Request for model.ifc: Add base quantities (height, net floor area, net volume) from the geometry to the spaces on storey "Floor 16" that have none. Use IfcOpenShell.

First a look at what the model holds.

```python
import ifcopenshell
import ifcopenshell.util.element
import ifcopenshell.util.unit

model = ifcopenshell.open("model.ifc")
print(model.schema)
for unit_type in ("LENGTHUNIT", "AREAUNIT", "VOLUMEUNIT"):
    print(unit_type, ifcopenshell.util.unit.calculate_unit_scale(model, unit_type))
storey = next(s for s in model.by_type("IfcBuildingStorey") if s.Name == "Floor 16")
spaces = [e for e in ifcopenshell.util.element.get_decomposition(storey) if e.is_a("IfcSpace")]
for e in sorted(spaces, key=lambda e: e.id()):
    print(e.id(), e.is_a(), e.Name, list(ifcopenshell.util.element.get_psets(e, qtos_only=True)), sep=" | ")
```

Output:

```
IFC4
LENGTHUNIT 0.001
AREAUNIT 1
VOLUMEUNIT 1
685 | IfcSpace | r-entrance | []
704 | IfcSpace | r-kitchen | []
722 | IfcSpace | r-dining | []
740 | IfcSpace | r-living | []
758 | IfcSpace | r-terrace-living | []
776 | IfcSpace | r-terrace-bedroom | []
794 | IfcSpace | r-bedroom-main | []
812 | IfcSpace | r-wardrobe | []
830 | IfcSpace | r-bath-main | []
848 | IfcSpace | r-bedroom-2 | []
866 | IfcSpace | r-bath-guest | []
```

```python
import ifcopenshell
import ifcopenshell.api.pset
import ifcopenshell.geom
import ifcopenshell.util.element
import ifcopenshell.util.shape
import ifcopenshell.util.unit

model = ifcopenshell.open("model.ifc")
unit_scale = ifcopenshell.util.unit.calculate_unit_scale(model)
area_scale = ifcopenshell.util.unit.calculate_unit_scale(model, "AREAUNIT")
volume_scale = ifcopenshell.util.unit.calculate_unit_scale(model, "VOLUMEUNIT")
settings = ifcopenshell.geom.settings()

storey = next(s for s in model.by_type("IfcBuildingStorey") if s.Name == "Floor 16")
spaces = [e for e in ifcopenshell.util.element.get_decomposition(storey) if e.is_a("IfcSpace")]

for e in sorted(spaces, key=lambda e: e.id()):
    if ifcopenshell.util.element.get_psets(e, qtos_only=True, should_inherit=False):
        continue
    # Geometry comes back in metres, in the element's own axes.
    shape = ifcopenshell.geom.create_shape(settings, e)
    values = {
        "Height": ifcopenshell.util.shape.get_z(shape.geometry) / unit_scale,
        "NetFloorArea": ifcopenshell.util.shape.get_footprint_area(shape.geometry) / area_scale,
        "NetVolume": ifcopenshell.util.shape.get_volume(shape.geometry) / volume_scale,
    }
    qto = ifcopenshell.api.pset.add_qto(model, product=e, name="Qto_SpaceBaseQuantities")
    ifcopenshell.api.pset.edit_qto(model, qto=qto, properties=values)
    print(e.id(), {k: round(v, 3) for k, v in values.items()})

model.write("model_v2.ifc")
```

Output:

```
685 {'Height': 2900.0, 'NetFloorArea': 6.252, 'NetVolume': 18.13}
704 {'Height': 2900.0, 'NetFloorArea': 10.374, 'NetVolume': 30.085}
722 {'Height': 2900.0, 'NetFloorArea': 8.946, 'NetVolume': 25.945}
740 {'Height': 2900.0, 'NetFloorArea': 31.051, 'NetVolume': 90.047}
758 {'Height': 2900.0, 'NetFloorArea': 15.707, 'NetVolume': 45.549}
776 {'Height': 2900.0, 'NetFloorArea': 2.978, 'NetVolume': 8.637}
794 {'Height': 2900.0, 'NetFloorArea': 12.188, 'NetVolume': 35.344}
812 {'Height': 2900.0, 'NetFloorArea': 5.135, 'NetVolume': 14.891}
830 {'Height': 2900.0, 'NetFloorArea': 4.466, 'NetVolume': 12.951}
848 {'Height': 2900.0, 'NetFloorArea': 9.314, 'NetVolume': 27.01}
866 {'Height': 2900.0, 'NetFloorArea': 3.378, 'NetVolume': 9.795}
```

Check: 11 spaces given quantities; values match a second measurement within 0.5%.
